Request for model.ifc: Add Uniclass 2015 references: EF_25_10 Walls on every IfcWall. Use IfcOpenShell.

First a look at what the model holds.

```python
import ifcopenshell

model = ifcopenshell.open("model.ifc")
print(model.schema)
print("classifications:", [c.Name for c in model.by_type("IfcClassification")])
for ifc_class in ("IfcDoor", "IfcRoof", "IfcStair", "IfcWall", "IfcWindow"):
    print(ifc_class, len(model.by_type(ifc_class)))
```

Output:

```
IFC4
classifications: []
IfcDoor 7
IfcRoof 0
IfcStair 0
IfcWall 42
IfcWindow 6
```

```python
import ifcopenshell
import ifcopenshell.api.classification

model = ifcopenshell.open("model.ifc")

system = ifcopenshell.api.classification.add_classification(model, classification="Uniclass 2015")

codes = {
    "IfcWall": ("EF_25_10", "Walls"),
}
for ifc_class, (code, name) in codes.items():
    products = model.by_type(ifc_class)
    ifcopenshell.api.classification.add_reference(
        model, products=products, classification=system, identification=code, name=name
    )
    print(code, len(products))

model.write("model_updated.ifc")
```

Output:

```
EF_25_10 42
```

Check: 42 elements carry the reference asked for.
